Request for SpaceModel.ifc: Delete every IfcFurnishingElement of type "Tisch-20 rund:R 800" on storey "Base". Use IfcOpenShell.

First a look at what the model holds.

```python
import ifcopenshell
import ifcopenshell.util.element

model = ifcopenshell.open("SpaceModel.ifc")
print(model.schema)
storey = next(s for s in model.by_type("IfcBuildingStorey") if s.Name == "Base")
furniture = [e for e in ifcopenshell.util.element.get_decomposition(storey) if e.is_a("IfcFurnishingElement")]
seen = {}
for e in furniture:
    element_type = ifcopenshell.util.element.get_type(e)
    name = element_type.Name if element_type not in (None, e) else None
    seen[name] = seen.get(name, 0) + 1
for name, count in sorted(seen.items(), key=str):
    print(count, "x", name)
```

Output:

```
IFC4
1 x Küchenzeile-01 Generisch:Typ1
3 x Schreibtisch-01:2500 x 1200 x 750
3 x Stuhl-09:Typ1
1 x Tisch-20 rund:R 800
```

```python
import ifcopenshell
import ifcopenshell.api.root
import ifcopenshell.util.element

model = ifcopenshell.open("SpaceModel.ifc")

storey = next(s for s in model.by_type("IfcBuildingStorey") if s.Name == "Base")
furniture = [e for e in ifcopenshell.util.element.get_decomposition(storey) if e.is_a("IfcFurnishingElement")]
targets = [e for e in furniture if (t := ifcopenshell.util.element.get_type(e)) not in (None, e) and t.Name == "Tisch-20 rund:R 800"]

for e in targets:
    ifcopenshell.api.root.remove_product(model, product=e)
print(len(targets), "removed")

model.write("SpaceModel_updated.ifc")
```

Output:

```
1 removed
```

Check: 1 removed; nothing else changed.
